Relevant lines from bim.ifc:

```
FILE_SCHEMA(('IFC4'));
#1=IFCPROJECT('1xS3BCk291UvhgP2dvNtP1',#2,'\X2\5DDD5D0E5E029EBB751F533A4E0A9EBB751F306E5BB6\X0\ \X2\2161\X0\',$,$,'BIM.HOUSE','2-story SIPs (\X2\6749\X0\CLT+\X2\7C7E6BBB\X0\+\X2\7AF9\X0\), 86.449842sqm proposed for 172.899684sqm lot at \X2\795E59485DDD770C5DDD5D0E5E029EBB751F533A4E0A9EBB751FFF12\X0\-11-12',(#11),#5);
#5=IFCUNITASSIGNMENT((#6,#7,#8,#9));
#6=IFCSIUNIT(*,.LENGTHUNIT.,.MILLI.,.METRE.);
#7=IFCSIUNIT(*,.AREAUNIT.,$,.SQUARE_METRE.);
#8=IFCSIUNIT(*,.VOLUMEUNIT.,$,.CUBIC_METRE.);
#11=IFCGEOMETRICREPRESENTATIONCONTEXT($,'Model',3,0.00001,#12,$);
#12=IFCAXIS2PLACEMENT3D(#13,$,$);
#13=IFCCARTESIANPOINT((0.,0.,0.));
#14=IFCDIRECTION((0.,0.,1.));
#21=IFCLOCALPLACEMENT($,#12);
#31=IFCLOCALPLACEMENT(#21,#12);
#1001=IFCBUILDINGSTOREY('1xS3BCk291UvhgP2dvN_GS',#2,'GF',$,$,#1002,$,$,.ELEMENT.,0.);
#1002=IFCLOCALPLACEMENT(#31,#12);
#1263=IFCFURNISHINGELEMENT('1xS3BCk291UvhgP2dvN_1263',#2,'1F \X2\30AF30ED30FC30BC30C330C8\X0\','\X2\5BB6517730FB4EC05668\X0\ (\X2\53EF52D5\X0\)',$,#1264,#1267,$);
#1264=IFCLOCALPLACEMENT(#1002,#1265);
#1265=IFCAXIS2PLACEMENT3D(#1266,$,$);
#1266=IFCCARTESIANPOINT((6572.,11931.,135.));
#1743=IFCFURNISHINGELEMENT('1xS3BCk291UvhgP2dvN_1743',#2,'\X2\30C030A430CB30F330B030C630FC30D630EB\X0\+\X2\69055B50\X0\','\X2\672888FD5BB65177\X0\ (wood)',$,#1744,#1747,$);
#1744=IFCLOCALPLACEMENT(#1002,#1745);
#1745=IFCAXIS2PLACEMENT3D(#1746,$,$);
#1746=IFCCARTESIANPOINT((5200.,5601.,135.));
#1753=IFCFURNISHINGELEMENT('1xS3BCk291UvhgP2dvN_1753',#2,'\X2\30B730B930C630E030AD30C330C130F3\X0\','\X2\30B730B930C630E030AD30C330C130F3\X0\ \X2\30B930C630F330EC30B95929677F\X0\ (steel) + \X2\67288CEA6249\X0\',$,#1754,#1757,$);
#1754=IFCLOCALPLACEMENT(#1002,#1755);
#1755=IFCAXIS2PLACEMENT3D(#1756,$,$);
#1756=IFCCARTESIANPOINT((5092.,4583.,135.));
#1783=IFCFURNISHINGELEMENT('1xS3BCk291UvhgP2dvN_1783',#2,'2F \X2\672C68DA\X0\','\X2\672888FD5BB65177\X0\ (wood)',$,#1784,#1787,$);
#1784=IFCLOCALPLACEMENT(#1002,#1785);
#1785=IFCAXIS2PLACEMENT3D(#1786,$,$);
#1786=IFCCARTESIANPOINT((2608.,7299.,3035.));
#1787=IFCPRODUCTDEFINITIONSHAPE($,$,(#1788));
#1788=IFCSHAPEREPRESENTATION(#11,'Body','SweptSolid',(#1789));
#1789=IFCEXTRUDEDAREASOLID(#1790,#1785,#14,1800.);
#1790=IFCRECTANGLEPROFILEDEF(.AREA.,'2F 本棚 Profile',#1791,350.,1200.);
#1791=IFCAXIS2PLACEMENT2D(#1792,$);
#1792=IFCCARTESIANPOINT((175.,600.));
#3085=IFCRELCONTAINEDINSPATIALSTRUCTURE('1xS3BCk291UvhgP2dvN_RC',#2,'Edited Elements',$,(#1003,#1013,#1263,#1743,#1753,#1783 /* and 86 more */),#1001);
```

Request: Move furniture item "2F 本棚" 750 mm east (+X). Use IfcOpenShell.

```python
import ifcopenshell
import ifcopenshell.api.geometry
import ifcopenshell.util.placement
import ifcopenshell.util.unit

model = ifcopenshell.open("bim.ifc")
unit_scale = ifcopenshell.util.unit.calculate_unit_scale(model)

item = model.by_guid("1xS3BCk291UvhgP2dvN_1783")
matrix = ifcopenshell.util.placement.get_local_placement(item.ObjectPlacement)
matrix[0, 3] += 0.75 / unit_scale
ifcopenshell.api.geometry.edit_object_placement(model, product=item, matrix=matrix, is_si=False)

print(ifcopenshell.util.placement.get_local_placement(item.ObjectPlacement).round(3) + 0.0)

model.write("bim_rev.ifc")
```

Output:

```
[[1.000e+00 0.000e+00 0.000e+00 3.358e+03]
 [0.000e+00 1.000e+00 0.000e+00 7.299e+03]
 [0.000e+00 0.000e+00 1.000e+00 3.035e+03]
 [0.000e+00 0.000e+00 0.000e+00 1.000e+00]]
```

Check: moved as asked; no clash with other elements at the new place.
